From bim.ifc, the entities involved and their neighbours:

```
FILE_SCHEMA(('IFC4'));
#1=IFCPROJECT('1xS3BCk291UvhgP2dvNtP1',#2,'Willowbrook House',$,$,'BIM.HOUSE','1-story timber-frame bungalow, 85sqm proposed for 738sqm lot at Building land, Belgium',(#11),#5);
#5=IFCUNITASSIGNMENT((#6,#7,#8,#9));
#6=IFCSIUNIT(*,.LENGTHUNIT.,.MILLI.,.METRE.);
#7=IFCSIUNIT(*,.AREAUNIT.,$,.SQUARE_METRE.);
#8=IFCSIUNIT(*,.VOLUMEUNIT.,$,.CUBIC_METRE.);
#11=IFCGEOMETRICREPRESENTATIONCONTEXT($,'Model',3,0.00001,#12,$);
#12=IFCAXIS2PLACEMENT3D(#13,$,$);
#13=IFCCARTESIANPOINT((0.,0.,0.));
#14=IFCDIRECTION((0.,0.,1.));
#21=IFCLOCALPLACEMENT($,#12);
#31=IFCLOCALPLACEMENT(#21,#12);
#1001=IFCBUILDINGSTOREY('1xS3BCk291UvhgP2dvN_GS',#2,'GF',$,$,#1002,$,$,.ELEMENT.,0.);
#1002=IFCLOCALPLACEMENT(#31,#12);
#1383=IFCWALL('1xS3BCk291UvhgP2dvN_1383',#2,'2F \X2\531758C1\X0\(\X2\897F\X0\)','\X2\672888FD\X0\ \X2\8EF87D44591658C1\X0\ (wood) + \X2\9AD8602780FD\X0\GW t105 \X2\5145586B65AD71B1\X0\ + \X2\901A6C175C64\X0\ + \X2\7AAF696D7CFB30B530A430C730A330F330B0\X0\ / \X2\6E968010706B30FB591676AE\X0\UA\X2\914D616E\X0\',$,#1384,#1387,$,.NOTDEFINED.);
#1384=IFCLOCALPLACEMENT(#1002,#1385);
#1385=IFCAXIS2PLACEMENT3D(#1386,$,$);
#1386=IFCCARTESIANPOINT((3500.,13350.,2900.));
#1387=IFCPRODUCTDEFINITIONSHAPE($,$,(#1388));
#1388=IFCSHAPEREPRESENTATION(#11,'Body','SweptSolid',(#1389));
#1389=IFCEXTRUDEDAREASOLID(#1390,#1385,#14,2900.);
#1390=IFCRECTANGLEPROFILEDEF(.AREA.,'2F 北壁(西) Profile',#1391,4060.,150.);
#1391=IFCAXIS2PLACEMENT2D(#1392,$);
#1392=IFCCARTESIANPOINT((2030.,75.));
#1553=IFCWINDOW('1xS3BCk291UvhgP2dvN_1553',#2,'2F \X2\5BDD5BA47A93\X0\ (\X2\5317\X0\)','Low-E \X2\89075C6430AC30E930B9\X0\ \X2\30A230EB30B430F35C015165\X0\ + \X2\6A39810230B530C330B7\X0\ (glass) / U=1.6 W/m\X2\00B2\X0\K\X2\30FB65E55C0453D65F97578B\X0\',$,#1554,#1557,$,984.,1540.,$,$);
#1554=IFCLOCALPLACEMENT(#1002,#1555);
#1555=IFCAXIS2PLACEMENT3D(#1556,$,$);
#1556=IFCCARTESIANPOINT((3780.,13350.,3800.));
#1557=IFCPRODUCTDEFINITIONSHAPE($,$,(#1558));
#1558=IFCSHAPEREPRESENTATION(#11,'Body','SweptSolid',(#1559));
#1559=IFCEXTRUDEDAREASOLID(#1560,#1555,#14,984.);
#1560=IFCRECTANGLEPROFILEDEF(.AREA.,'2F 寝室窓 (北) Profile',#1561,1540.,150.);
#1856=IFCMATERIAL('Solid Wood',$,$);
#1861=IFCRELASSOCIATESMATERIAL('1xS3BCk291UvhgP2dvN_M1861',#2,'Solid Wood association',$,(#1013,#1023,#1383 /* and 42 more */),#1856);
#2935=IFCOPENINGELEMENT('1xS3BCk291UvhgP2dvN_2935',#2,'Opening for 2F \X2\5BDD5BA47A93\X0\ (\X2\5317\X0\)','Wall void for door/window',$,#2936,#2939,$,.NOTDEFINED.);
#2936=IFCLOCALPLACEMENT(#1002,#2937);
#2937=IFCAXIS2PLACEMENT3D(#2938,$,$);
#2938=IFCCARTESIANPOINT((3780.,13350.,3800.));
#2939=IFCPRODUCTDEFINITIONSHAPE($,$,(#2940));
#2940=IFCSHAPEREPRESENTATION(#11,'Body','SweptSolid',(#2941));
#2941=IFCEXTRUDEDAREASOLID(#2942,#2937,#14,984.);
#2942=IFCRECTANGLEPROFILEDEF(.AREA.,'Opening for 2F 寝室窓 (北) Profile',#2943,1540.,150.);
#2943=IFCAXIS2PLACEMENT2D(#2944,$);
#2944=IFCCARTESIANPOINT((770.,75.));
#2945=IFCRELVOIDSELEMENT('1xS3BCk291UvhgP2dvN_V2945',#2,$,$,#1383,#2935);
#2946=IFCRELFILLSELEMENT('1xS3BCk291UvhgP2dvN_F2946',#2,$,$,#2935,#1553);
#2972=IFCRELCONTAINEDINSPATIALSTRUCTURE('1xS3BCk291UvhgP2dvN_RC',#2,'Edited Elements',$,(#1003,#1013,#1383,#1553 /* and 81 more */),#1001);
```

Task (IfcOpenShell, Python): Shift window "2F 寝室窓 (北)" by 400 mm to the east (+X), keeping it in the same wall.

```python
import ifcopenshell
import ifcopenshell.api.geometry
import ifcopenshell.util.placement
import ifcopenshell.util.unit

model = ifcopenshell.open("bim.ifc")
unit_scale = ifcopenshell.util.unit.calculate_unit_scale(model)

window = model.by_guid("1xS3BCk291UvhgP2dvN_1553")
opening = window.FillsVoids[0].RelatingOpeningElement
wall = opening.VoidsElements[0].RelatingBuildingElement

wall_matrix = ifcopenshell.util.placement.get_local_placement(wall.ObjectPlacement)
shift = wall_matrix[:3, 0] * 0.4 / unit_scale
before = ifcopenshell.util.placement.get_local_placement(window.ObjectPlacement)[:3, 3].copy()

# The window is not placed relative to its opening, so move both.
for product in (opening, window):
    matrix = ifcopenshell.util.placement.get_local_placement(product.ObjectPlacement)
    matrix[:3, 3] += shift
    ifcopenshell.api.geometry.edit_object_placement(model, product=product, matrix=matrix, is_si=False)

after = ifcopenshell.util.placement.get_local_placement(window.ObjectPlacement)[:3, 3]
print("window moved by", (after - before).round(3) + 0.0)

model.write("bim_rev.ifc")
```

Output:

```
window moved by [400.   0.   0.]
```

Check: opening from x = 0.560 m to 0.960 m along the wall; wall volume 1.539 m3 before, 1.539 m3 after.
